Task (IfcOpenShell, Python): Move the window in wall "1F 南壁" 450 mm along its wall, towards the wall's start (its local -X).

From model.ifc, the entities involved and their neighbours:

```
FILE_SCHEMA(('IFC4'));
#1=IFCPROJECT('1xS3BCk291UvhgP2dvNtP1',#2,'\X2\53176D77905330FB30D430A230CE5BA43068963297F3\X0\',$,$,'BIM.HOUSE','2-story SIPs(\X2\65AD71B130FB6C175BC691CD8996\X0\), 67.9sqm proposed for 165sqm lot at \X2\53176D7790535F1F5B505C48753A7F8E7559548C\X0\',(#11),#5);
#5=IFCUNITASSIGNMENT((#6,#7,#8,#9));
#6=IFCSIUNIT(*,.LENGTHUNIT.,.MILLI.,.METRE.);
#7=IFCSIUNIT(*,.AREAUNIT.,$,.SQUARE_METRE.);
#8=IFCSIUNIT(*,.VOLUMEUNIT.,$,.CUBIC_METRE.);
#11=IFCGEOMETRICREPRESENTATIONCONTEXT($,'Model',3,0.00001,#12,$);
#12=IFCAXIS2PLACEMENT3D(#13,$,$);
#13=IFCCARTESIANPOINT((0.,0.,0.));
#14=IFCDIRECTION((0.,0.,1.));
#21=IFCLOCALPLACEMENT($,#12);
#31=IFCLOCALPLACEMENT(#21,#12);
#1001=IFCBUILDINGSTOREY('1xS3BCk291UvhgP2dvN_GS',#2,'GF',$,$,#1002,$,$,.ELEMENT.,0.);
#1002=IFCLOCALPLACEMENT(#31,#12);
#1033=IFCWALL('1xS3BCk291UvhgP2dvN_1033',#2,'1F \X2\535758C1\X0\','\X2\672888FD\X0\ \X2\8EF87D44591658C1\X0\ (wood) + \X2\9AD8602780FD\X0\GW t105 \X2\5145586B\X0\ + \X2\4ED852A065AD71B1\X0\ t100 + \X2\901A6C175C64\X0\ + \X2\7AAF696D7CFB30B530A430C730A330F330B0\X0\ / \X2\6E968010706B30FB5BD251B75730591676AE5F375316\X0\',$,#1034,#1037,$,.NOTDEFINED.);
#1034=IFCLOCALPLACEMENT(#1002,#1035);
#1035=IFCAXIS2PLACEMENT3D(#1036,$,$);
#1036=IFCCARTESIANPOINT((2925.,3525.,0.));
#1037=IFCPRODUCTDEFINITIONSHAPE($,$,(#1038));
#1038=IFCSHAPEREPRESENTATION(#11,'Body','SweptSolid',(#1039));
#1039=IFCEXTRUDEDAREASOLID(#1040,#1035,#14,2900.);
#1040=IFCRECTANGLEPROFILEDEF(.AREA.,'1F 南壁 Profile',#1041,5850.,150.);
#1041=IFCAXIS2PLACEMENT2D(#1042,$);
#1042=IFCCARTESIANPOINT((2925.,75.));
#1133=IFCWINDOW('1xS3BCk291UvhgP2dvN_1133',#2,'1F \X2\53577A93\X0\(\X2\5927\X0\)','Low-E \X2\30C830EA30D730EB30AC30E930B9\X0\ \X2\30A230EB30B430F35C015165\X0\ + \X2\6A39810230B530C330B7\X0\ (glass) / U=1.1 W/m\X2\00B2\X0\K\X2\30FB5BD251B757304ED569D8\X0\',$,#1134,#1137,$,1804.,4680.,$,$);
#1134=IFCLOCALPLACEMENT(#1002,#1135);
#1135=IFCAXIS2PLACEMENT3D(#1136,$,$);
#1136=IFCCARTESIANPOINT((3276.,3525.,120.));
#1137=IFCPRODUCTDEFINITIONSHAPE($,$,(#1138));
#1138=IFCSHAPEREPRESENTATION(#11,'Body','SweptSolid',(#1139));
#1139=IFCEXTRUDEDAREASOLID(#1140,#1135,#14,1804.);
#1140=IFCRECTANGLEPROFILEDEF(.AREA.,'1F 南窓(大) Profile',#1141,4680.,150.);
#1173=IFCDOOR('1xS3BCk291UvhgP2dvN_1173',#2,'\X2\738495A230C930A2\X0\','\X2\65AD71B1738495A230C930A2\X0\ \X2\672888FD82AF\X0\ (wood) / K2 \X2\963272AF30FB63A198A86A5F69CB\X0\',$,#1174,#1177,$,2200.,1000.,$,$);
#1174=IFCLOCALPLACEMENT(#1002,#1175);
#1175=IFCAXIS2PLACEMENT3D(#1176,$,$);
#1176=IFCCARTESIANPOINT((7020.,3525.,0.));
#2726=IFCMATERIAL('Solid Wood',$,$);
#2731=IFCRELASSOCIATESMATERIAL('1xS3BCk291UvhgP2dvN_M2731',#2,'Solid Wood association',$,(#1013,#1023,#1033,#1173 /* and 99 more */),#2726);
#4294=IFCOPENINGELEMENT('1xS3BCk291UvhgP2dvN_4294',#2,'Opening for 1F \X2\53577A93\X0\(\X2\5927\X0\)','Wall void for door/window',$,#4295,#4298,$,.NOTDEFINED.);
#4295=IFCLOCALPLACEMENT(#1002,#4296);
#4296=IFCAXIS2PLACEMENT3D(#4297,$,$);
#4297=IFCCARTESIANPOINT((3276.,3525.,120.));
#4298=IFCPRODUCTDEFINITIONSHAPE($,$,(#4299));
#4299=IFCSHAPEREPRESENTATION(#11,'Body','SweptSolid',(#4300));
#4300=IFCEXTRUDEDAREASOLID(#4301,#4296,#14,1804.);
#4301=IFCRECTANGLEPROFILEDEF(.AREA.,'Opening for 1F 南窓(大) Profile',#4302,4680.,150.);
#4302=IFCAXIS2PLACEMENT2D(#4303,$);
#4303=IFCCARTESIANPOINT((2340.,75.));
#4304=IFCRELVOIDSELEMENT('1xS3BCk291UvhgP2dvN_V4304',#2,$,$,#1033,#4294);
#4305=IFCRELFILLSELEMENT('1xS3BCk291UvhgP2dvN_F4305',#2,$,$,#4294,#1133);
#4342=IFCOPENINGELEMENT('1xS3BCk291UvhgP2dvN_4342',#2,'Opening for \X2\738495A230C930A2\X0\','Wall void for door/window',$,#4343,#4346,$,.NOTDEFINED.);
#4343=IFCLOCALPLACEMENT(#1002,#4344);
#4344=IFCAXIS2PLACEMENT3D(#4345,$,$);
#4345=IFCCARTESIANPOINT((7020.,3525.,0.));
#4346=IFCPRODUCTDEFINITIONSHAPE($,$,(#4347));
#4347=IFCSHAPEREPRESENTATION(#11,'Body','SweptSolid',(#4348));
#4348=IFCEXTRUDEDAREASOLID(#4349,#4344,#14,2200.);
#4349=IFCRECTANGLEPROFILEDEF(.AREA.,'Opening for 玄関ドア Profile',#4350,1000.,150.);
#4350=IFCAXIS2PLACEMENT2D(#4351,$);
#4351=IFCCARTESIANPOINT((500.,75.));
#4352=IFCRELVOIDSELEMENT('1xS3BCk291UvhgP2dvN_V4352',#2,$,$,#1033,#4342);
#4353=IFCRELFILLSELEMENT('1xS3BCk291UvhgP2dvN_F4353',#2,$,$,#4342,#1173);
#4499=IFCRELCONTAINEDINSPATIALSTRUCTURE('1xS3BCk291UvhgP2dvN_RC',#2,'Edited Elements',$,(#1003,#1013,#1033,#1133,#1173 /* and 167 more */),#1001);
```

```python
import ifcopenshell
import ifcopenshell.api.geometry
import ifcopenshell.util.placement
import ifcopenshell.util.unit

model = ifcopenshell.open("model.ifc")
unit_scale = ifcopenshell.util.unit.calculate_unit_scale(model)

window = model.by_guid("1xS3BCk291UvhgP2dvN_1133")
opening = window.FillsVoids[0].RelatingOpeningElement
wall = opening.VoidsElements[0].RelatingBuildingElement

wall_matrix = ifcopenshell.util.placement.get_local_placement(wall.ObjectPlacement)
shift = wall_matrix[:3, 0] * -0.45 / unit_scale
before = ifcopenshell.util.placement.get_local_placement(window.ObjectPlacement)[:3, 3].copy()

# The window is not placed relative to its opening, so move both.
for product in (opening, window):
    matrix = ifcopenshell.util.placement.get_local_placement(product.ObjectPlacement)
    matrix[:3, 3] += shift
    ifcopenshell.api.geometry.edit_object_placement(model, product=product, matrix=matrix, is_si=False)

after = ifcopenshell.util.placement.get_local_placement(window.ObjectPlacement)[:3, 3]
print("window moved by", (after - before).round(3) + 0.0)

model.write("model_v2.ifc")
```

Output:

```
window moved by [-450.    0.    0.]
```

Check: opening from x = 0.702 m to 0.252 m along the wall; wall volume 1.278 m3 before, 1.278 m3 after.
